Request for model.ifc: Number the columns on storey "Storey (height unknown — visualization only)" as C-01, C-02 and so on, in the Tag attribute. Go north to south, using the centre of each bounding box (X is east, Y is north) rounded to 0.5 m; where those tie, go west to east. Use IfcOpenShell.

First a look at what the model holds.

```python
import ifcopenshell
import ifcopenshell.util.element
import ifcopenshell.util.placement

model = ifcopenshell.open("model.ifc")
print(model.schema)
storey = next(s for s in model.by_type("IfcBuildingStorey") if s.Name == "Storey (height unknown — visualization only)")
columns = [e for e in ifcopenshell.util.element.get_decomposition(storey) if e.is_a("IfcColumn")]
for e in sorted(columns, key=lambda e: e.id()):
    origin = ifcopenshell.util.placement.get_local_placement(e.ObjectPlacement)[:3, 3]
    print(e.id(), e.Tag, e.Name, origin.round(2) + 0.0, sep=" | ")
```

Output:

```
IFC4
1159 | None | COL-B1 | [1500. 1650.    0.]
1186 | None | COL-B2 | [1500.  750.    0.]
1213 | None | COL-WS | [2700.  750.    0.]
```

```python
import ifcopenshell
import ifcopenshell.geom
import ifcopenshell.util.element
import ifcopenshell.util.shape

model = ifcopenshell.open("model.ifc")
settings = ifcopenshell.geom.settings()
settings.set("use-world-coords", True)


def centre(element):
    shape = ifcopenshell.geom.create_shape(settings, element)
    return ifcopenshell.util.shape.get_bbox_centroid(shape.geometry)


storey = next(s for s in model.by_type("IfcBuildingStorey") if s.Name == "Storey (height unknown — visualization only)")
columns = [e for e in ifcopenshell.util.element.get_decomposition(storey) if e.is_a("IfcColumn")]

# Insertion points can sit at a corner or the storey origin, so sort by the geometry (in metres).
centres = {e: centre(e) for e in columns}
columns.sort(key=lambda e: (-round(centres[e][1] / 0.5), centres[e][0]))

for i, e in enumerate(columns, start=1):
    number = f"C-{i:02d}"
    e.Tag = number
    print(e.id(), number)

model.write("model_edited.ifc")
```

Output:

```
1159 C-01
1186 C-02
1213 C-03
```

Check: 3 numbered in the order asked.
